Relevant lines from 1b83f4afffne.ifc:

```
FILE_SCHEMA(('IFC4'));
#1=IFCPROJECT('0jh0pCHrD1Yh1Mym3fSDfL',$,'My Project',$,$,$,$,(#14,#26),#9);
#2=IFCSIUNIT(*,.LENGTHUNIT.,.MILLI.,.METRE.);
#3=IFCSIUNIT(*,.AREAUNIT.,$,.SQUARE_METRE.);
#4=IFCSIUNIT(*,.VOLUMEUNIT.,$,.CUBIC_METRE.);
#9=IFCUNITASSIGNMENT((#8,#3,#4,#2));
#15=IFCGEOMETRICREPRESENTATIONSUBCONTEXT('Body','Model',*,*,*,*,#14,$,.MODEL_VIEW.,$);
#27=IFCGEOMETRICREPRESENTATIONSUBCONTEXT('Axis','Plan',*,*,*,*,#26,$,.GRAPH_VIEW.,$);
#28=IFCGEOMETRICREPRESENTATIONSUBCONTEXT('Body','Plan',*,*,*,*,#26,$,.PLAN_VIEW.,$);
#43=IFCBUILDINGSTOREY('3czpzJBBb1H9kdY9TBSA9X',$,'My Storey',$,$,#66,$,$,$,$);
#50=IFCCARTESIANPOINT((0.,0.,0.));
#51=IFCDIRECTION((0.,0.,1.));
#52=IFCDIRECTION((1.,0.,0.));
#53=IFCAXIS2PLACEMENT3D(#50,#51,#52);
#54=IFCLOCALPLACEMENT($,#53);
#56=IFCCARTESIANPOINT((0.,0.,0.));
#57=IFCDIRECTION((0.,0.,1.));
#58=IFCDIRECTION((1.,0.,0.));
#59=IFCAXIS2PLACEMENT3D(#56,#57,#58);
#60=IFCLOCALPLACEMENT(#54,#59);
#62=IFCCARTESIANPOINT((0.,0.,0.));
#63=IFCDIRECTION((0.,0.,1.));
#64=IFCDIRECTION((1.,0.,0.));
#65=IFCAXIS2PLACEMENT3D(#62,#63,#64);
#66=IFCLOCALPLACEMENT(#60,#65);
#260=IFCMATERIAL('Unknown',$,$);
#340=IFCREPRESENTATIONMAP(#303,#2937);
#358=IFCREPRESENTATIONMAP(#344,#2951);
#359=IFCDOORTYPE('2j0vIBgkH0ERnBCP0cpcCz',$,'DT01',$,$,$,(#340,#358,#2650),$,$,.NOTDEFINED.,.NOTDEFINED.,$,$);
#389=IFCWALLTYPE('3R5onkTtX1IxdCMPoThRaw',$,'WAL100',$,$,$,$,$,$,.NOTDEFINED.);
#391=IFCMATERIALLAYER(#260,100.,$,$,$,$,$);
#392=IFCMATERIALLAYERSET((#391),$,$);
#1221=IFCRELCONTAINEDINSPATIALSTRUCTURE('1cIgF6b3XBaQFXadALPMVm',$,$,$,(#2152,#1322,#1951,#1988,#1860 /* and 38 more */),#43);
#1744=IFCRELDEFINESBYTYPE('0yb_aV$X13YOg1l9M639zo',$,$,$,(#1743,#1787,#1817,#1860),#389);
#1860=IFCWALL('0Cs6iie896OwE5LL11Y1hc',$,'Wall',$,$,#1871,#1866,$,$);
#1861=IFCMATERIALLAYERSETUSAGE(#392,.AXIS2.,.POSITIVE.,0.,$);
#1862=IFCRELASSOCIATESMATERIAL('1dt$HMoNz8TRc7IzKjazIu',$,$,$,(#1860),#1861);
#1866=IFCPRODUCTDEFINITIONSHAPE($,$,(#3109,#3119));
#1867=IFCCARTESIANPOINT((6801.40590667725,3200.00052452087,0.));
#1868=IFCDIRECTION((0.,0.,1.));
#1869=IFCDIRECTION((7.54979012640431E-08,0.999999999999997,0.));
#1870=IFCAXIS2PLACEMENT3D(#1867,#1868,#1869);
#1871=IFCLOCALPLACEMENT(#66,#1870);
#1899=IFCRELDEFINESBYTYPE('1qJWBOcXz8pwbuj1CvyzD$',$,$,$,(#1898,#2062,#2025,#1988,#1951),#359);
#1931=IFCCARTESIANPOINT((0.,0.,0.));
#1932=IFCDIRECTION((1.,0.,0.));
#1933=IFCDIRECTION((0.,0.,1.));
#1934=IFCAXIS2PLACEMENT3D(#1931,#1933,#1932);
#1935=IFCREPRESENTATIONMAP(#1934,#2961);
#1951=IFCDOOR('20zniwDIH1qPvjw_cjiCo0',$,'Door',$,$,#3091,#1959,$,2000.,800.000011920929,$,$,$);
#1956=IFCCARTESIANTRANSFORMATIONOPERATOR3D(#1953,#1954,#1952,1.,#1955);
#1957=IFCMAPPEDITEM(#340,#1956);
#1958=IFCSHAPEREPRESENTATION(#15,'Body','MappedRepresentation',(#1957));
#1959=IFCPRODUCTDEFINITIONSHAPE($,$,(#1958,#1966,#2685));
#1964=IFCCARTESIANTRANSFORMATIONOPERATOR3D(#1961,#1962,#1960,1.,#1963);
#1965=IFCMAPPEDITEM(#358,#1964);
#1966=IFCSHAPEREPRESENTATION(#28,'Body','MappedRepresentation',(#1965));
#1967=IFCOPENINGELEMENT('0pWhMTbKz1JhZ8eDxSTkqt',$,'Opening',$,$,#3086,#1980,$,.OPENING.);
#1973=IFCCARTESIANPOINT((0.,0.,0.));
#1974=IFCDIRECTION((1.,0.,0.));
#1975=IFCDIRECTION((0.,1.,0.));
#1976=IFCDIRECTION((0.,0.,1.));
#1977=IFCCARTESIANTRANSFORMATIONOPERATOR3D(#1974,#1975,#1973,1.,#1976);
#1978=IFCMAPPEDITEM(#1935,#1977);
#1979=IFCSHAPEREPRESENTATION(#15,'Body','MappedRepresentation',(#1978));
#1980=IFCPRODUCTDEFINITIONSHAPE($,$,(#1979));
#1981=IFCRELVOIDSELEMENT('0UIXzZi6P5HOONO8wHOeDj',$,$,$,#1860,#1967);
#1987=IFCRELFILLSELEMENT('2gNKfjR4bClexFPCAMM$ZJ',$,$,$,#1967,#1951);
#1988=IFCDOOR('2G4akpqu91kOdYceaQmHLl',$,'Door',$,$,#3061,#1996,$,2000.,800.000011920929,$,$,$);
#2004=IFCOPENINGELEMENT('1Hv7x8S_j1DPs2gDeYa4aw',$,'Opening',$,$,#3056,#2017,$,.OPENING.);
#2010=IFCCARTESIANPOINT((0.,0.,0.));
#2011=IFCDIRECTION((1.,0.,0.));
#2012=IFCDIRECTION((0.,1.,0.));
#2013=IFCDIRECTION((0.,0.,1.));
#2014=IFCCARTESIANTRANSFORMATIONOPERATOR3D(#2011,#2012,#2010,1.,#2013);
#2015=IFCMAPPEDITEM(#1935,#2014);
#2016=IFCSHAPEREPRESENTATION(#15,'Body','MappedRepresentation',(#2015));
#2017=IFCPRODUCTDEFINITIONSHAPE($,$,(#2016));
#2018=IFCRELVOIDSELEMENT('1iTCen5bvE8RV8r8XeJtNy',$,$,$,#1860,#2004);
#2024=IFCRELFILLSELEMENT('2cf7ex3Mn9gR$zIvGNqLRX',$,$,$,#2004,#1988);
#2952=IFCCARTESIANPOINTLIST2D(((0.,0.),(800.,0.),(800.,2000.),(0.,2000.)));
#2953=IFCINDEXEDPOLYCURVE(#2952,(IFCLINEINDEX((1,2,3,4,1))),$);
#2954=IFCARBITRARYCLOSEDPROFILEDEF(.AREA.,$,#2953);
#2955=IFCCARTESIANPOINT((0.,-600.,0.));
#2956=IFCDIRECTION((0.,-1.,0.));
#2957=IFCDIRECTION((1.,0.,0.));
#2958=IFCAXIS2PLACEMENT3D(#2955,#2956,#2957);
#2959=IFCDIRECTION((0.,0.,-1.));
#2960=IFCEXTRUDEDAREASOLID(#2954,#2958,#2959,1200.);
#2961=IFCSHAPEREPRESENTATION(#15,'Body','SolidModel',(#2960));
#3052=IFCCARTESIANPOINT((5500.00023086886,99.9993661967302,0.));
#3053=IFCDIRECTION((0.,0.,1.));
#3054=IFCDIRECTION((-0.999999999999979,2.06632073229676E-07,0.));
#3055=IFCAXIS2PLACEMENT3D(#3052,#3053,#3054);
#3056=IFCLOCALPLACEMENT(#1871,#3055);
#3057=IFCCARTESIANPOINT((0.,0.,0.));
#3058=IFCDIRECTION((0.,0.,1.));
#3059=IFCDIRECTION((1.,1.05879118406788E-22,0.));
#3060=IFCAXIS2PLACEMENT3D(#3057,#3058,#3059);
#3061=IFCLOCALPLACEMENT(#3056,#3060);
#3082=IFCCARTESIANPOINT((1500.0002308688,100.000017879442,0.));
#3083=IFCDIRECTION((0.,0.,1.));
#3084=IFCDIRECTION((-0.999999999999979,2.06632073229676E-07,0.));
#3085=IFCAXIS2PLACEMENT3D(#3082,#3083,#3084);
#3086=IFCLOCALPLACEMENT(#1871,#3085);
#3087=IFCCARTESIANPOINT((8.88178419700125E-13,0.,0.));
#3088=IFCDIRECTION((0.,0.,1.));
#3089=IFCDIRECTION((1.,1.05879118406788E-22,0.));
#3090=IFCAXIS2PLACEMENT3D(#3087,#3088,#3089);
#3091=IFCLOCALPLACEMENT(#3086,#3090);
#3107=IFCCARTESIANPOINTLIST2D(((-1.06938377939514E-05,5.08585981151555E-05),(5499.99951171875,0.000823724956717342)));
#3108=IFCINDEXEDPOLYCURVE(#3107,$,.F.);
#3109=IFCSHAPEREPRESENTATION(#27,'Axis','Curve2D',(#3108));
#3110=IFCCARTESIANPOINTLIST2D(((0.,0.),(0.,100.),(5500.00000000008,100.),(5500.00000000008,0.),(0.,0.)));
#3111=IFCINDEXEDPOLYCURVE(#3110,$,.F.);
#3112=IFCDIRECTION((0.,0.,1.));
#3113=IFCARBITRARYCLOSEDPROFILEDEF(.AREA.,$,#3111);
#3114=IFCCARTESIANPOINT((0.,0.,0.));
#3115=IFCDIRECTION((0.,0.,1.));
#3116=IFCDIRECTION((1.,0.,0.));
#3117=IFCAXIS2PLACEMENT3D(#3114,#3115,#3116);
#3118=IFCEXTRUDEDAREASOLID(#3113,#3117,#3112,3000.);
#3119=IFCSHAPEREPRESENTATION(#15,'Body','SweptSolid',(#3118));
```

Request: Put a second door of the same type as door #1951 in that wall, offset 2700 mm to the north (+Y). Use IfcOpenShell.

```python
import ifcopenshell
import ifcopenshell.api.feature
import ifcopenshell.api.geometry
import ifcopenshell.api.root
import ifcopenshell.geom
import ifcopenshell.util.element
import ifcopenshell.util.placement
import ifcopenshell.util.shape

model = ifcopenshell.open("1b83f4afffne.ifc")
settings = ifcopenshell.geom.settings()


def volume(element):
    """Net volume in cubic metres, openings subtracted."""
    shape = ifcopenshell.geom.create_shape(settings, element)
    return ifcopenshell.util.shape.get_volume(shape.geometry)


door = model.by_id(1951)
opening = door.FillsVoids[0].RelatingOpeningElement
wall = opening.VoidsElements[0].RelatingBuildingElement
before = volume(wall)
shift = ifcopenshell.util.placement.get_local_placement(wall.ObjectPlacement)[:3, 0] * 2700.0

# copy_class copies the void relationship, type, container and properties, but no geometry.
new_opening = ifcopenshell.api.root.copy_class(model, product=opening)
new_opening.Representation = ifcopenshell.util.element.copy_deep(
    model, opening.Representation, exclude=["IfcGeometricRepresentationContext", "IfcRepresentationMap"]
)
new_door = ifcopenshell.api.root.copy_class(model, product=door)
new_door.Representation = ifcopenshell.util.element.copy_deep(
    model, door.Representation, exclude=["IfcGeometricRepresentationContext", "IfcRepresentationMap"]
)
ifcopenshell.api.feature.add_filling(model, opening=new_opening, element=new_door)

for old, new in ((opening, new_opening), (door, new_door)):
    matrix = ifcopenshell.util.placement.get_local_placement(old.ObjectPlacement)
    matrix[:3, 3] += shift
    ifcopenshell.api.geometry.edit_object_placement(model, product=new, matrix=matrix, is_si=False)

after = volume(wall)

print(f"wall volume {before:.3f} -> {after:.3f} m3")

model.write("1b83f4afffne-out.ifc")
```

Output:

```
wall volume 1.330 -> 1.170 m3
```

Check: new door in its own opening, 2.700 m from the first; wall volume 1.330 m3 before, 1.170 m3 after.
